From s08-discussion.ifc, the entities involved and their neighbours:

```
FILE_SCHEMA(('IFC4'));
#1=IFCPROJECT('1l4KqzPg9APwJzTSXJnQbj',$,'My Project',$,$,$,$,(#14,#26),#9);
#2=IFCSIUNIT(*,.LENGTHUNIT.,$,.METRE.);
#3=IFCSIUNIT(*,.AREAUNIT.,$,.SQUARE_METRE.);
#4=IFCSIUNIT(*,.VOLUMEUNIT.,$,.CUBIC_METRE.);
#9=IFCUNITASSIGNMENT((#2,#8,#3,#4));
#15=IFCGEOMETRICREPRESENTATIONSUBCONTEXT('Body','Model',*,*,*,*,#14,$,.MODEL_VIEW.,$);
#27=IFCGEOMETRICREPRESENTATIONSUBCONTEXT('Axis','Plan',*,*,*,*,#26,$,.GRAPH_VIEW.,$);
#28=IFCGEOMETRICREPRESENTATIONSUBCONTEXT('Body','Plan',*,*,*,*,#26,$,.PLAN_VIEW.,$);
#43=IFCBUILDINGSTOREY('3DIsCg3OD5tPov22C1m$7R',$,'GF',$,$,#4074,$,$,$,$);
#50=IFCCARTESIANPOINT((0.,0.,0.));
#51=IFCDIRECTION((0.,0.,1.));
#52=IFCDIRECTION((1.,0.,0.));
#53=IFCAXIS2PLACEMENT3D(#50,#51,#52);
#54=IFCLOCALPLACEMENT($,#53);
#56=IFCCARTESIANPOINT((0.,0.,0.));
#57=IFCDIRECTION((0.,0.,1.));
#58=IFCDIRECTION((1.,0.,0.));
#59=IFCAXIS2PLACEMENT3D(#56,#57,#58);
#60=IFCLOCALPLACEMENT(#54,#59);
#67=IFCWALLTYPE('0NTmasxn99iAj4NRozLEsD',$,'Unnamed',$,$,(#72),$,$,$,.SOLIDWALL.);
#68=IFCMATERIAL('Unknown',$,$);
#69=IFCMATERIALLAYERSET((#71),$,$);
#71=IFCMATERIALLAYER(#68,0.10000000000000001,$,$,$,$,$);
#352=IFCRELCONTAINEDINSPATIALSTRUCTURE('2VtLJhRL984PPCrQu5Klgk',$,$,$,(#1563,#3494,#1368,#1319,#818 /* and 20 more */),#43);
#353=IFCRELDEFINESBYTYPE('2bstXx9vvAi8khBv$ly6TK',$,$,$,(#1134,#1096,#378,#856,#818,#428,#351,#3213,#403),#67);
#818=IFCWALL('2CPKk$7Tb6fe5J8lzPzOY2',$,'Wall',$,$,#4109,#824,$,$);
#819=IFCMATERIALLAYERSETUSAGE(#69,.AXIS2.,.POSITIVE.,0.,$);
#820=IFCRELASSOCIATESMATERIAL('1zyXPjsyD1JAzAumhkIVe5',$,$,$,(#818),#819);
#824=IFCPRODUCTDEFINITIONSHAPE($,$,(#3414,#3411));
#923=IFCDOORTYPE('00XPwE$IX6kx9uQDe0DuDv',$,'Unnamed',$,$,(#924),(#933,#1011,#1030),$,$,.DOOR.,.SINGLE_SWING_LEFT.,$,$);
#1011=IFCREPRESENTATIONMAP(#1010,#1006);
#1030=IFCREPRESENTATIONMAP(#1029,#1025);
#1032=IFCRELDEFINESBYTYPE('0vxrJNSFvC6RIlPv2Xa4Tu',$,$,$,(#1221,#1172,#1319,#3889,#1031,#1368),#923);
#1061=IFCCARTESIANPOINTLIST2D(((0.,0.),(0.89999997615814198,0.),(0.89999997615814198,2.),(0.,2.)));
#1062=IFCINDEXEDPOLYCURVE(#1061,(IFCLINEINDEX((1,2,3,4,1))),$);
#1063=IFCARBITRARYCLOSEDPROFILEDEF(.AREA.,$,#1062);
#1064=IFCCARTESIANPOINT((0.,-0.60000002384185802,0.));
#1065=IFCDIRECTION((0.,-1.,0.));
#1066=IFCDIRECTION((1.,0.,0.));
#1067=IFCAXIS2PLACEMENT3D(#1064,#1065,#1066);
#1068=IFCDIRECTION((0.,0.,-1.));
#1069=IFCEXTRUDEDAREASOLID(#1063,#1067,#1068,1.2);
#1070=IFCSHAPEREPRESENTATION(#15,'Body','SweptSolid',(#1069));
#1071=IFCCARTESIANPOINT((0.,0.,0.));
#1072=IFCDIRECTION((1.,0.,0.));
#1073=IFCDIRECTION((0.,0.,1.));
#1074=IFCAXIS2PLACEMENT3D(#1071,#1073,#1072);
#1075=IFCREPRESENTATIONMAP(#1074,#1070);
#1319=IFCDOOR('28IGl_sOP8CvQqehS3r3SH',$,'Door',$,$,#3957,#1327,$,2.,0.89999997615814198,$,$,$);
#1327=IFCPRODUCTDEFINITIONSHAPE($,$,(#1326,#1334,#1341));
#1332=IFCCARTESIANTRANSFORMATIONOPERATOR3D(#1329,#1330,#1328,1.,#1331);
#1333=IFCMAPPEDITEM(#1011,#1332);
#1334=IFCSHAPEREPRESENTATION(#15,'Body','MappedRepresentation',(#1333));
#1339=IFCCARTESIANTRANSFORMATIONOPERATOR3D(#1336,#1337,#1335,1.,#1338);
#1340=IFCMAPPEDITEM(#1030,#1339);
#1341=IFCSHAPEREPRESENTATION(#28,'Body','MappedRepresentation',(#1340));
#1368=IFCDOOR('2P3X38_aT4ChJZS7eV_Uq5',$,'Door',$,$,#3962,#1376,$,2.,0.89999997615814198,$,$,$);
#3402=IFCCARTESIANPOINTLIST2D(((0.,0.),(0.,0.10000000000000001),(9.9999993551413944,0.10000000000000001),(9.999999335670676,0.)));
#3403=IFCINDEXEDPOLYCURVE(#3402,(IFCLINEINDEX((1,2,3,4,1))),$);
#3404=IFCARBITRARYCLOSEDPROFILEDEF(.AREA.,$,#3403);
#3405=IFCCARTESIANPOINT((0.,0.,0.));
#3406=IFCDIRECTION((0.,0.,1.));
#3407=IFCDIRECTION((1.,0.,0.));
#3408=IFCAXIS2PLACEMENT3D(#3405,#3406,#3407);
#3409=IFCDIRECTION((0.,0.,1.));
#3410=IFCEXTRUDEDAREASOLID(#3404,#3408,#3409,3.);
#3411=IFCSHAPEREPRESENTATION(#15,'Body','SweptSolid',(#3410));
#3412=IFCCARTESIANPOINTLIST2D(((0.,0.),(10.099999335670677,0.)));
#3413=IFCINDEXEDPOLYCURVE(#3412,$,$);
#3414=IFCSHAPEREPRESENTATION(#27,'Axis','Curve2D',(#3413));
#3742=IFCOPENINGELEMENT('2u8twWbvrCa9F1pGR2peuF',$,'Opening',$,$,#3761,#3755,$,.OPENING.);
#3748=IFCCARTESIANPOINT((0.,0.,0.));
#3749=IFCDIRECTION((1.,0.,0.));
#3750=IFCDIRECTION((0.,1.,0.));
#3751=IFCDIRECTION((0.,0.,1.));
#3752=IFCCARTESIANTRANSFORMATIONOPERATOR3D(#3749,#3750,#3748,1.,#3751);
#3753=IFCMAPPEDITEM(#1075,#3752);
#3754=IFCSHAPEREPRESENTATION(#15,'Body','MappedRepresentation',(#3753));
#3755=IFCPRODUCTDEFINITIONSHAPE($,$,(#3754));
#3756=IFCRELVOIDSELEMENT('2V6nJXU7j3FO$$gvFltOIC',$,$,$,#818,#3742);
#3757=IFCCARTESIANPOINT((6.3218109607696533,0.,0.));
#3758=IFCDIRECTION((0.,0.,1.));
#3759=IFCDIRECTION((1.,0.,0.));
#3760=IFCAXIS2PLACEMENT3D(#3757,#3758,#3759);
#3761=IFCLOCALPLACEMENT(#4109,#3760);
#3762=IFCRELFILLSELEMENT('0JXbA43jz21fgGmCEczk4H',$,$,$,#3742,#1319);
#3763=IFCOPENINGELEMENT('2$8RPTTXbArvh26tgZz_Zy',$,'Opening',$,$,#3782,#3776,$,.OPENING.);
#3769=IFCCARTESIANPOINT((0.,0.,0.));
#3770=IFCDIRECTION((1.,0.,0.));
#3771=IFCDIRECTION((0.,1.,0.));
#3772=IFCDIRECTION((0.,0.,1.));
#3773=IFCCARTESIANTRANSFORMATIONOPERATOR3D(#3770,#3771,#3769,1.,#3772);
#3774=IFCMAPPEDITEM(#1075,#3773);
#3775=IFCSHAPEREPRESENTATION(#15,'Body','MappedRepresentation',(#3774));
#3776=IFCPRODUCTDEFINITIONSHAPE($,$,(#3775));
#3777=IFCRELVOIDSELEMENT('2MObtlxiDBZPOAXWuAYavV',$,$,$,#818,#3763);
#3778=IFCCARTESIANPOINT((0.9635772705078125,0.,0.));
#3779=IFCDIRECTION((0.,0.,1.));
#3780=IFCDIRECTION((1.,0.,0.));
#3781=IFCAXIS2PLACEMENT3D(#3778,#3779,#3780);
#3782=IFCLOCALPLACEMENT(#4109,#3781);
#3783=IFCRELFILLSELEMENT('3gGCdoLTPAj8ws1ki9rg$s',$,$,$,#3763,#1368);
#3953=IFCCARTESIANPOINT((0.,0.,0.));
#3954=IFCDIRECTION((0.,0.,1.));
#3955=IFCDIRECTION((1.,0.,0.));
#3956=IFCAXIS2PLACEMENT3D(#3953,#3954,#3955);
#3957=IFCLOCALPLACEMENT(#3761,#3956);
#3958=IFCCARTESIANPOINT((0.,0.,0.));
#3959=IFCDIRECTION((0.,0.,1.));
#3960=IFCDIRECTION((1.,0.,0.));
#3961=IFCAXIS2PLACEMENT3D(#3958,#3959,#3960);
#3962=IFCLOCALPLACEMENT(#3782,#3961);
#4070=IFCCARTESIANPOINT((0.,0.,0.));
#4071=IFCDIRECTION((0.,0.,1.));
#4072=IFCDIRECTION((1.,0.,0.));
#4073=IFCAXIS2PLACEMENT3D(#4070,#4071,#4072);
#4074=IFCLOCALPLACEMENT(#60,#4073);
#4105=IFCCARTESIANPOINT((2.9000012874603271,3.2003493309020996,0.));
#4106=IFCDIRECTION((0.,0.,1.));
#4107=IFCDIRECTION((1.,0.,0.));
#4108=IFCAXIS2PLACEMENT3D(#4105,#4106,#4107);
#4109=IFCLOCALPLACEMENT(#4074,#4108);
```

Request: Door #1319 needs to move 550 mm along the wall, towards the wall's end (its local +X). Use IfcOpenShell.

```python
import ifcopenshell
import ifcopenshell.api.geometry
import ifcopenshell.util.placement
import ifcopenshell.util.unit

model = ifcopenshell.open("s08-discussion.ifc")
unit_scale = ifcopenshell.util.unit.calculate_unit_scale(model)

door = model.by_id(1319)
opening = door.FillsVoids[0].RelatingOpeningElement
wall = opening.VoidsElements[0].RelatingBuildingElement

wall_matrix = ifcopenshell.util.placement.get_local_placement(wall.ObjectPlacement)
shift = wall_matrix[:3, 0] * 0.55 / unit_scale
before = ifcopenshell.util.placement.get_local_placement(door.ObjectPlacement)[:3, 3].copy()

# The door is placed relative to its opening, so it follows when the opening moves.
matrix = ifcopenshell.util.placement.get_local_placement(opening.ObjectPlacement)
matrix[:3, 3] += shift
ifcopenshell.api.geometry.edit_object_placement(
    model, product=opening, matrix=matrix, is_si=False, should_transform_children=True
)

after = ifcopenshell.util.placement.get_local_placement(door.ObjectPlacement)[:3, 3]
print("door moved by", (after - before).round(3) + 0.0)

model.write("s08-discussion_v2.ifc")
```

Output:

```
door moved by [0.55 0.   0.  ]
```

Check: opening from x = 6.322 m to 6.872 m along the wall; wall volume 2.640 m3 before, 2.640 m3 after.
